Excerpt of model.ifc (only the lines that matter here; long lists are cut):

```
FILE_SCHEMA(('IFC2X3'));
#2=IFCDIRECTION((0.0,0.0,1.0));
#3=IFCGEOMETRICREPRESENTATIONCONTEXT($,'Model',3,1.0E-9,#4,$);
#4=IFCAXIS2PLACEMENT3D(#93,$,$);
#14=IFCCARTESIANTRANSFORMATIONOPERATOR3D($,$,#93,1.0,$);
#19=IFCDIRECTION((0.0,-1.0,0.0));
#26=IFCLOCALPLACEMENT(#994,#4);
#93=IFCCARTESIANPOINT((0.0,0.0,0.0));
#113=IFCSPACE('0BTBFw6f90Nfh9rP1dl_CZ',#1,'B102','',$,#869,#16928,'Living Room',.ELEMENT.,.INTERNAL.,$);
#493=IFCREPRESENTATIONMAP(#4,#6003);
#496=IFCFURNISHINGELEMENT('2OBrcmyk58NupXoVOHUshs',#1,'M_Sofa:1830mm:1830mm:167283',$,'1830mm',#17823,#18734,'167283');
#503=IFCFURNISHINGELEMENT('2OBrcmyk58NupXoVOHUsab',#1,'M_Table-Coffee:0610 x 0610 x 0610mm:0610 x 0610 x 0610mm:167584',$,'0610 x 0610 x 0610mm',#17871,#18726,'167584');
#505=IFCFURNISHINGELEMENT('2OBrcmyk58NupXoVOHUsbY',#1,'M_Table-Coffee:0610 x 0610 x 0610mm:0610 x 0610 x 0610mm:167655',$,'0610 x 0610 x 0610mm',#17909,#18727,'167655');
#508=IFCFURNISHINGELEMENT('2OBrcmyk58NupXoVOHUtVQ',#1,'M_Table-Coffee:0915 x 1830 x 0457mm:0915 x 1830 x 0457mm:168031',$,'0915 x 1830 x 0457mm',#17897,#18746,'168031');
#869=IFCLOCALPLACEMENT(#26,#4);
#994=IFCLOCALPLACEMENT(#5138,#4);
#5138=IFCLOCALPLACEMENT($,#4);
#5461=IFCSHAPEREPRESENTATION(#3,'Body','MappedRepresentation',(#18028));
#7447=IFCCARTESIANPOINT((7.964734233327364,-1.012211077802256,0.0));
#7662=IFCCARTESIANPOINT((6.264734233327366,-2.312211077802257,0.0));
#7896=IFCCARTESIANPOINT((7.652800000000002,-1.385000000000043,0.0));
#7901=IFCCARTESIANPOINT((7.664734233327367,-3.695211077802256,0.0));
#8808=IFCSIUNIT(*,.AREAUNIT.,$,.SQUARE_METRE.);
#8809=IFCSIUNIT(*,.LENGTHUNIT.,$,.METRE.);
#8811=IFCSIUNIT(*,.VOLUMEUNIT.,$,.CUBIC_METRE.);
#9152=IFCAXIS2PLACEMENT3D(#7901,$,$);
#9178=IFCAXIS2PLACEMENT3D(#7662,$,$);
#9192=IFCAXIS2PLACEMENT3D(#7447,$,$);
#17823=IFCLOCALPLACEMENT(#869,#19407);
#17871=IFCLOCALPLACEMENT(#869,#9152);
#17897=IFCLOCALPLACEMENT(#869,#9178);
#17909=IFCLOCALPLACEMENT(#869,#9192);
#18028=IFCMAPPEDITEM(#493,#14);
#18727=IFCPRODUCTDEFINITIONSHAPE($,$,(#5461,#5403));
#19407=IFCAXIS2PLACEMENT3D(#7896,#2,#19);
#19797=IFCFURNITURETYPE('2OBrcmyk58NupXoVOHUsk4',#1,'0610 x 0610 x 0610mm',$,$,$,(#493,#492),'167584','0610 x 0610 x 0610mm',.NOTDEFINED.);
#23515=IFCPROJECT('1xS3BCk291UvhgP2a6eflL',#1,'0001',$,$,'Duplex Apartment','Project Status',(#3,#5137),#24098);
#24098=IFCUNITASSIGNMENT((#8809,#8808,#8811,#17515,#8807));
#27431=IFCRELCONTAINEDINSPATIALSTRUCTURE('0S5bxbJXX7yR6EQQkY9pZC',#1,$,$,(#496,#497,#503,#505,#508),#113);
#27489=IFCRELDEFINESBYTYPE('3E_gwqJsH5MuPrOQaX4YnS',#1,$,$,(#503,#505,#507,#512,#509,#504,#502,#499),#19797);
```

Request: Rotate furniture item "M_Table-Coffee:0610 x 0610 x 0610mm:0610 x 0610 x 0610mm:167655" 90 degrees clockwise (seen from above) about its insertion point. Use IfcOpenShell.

```python
import ifcopenshell
import ifcopenshell.api.geometry
import ifcopenshell.util.placement

model = ifcopenshell.open("model.ifc")

item = model.by_id(505)
matrix = ifcopenshell.util.placement.get_local_placement(item.ObjectPlacement)
matrix = matrix @ ifcopenshell.util.placement.rotation(-90, "Z")
ifcopenshell.api.geometry.edit_object_placement(model, product=item, matrix=matrix, is_si=False)

print(ifcopenshell.util.placement.get_local_placement(item.ObjectPlacement).round(3) + 0.0)

model.write("model_v2.ifc")
```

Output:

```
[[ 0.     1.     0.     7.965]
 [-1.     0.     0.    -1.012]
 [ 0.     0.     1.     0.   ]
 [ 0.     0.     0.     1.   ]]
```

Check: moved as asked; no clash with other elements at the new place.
